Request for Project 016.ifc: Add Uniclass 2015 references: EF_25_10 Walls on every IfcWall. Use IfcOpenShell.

First a look at what the model holds.

```python
import ifcopenshell

model = ifcopenshell.open("Project 016.ifc")
print(model.schema)
print("classifications:", [c.Name for c in model.by_type("IfcClassification")])
for ifc_class in ("IfcDoor", "IfcRoof", "IfcStair", "IfcWall", "IfcWindow"):
    print(ifc_class, len(model.by_type(ifc_class)))
```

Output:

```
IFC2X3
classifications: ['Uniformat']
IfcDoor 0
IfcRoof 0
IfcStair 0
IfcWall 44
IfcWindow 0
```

```python
import ifcopenshell
import ifcopenshell.api.classification

model = ifcopenshell.open("Project 016.ifc")

# IFC2X3 requires Source and Edition and has no link from the project to the system.
system = model.create_entity("IfcClassification", Source="NBS", Edition="2015", Name="Uniclass 2015")

codes = {
    "IfcWall": ("EF_25_10", "Walls"),
}
for ifc_class, (code, name) in codes.items():
    products = model.by_type(ifc_class)
    ifcopenshell.api.classification.add_reference(
        model, products=products, classification=system, identification=code, name=name
    )
    print(code, len(products))

model.write("Project 016_updated.ifc")
```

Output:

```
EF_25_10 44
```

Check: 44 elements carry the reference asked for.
